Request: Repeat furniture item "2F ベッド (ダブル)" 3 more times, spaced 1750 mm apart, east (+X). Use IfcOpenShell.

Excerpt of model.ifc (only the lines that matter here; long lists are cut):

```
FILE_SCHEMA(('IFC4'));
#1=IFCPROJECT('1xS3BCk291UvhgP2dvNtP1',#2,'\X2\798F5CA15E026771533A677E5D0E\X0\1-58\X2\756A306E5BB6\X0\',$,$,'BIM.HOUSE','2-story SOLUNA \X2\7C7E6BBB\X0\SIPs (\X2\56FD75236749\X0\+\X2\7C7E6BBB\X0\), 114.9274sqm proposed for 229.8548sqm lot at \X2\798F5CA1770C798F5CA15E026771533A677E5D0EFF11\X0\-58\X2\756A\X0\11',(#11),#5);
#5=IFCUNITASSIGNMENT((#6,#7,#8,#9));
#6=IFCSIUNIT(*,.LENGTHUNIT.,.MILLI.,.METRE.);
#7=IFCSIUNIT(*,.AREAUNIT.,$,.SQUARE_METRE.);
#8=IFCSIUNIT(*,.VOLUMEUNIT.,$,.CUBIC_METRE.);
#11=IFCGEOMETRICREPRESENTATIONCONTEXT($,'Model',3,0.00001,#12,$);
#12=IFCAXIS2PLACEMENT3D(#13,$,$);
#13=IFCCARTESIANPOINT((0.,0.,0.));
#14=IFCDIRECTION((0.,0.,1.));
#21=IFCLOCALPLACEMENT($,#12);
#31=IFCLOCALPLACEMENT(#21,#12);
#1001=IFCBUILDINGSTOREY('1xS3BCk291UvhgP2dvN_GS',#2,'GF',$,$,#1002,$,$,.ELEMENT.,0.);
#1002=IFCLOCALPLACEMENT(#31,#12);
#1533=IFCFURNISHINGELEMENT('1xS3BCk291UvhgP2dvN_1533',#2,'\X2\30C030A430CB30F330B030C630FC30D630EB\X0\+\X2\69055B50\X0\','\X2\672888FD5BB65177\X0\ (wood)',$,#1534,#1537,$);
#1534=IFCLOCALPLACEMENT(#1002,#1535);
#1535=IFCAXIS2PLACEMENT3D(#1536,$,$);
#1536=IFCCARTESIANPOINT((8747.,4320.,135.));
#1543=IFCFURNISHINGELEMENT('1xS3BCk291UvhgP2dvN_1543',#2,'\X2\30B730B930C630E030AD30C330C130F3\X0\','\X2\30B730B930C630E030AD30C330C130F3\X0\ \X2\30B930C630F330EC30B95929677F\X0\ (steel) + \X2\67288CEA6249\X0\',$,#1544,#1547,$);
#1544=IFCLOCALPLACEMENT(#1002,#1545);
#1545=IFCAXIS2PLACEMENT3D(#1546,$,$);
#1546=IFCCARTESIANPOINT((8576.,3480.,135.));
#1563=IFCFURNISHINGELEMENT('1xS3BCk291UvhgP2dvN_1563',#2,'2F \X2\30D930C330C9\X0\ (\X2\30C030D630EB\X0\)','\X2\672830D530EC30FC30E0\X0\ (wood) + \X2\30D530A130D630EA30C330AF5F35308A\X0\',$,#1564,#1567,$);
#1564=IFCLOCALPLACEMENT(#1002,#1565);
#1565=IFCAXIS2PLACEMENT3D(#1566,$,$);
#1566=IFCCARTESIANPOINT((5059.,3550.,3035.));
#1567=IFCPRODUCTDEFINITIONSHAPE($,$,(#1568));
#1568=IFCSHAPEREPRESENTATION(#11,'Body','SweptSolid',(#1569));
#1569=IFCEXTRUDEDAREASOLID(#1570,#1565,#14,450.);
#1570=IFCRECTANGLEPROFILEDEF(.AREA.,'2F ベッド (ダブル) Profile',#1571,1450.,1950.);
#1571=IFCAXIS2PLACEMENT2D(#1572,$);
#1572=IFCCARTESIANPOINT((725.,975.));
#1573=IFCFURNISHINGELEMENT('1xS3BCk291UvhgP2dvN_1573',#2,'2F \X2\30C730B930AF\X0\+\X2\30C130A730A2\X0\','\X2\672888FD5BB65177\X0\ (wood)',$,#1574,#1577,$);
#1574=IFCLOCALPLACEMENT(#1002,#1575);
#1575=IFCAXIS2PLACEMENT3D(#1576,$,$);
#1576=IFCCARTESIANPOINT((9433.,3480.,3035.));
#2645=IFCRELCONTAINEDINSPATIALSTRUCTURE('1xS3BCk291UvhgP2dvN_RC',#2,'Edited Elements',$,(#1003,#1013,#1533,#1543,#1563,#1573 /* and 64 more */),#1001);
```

```python
import numpy as np
import ifcopenshell
import ifcopenshell.api.geometry
import ifcopenshell.api.root
import ifcopenshell.util.element
import ifcopenshell.util.placement
import ifcopenshell.util.unit

model = ifcopenshell.open("model.ifc")
unit_scale = ifcopenshell.util.unit.calculate_unit_scale(model)


def reuse_history(source, copy):
    """copy_class also copies each property set's owner history, people and application; keep the originals."""
    for rel in copy.IsDefinedBy:
        if rel.is_a("IfcRelDefinesByProperties") and (history := rel.RelatingPropertyDefinition.OwnerHistory):
            rel.RelatingPropertyDefinition.OwnerHistory = source.OwnerHistory
            ifcopenshell.util.element.remove_deep2(model, history)


source = model.by_id(1563)
base = ifcopenshell.util.placement.get_local_placement(source.ObjectPlacement)
step = np.array([1.0, 0.0, 0.0]) * 1.75 / unit_scale

for i in range(1, 4):
    copy = ifcopenshell.api.root.copy_class(model, product=source)
    copy.Representation = ifcopenshell.util.element.copy_deep(
        model, source.Representation, exclude=["IfcGeometricRepresentationContext", "IfcRepresentationMap"]
    )
    reuse_history(source, copy)
    matrix = base.copy()
    matrix[:3, 3] += i * step
    print("added at", matrix[:3, 3].round(3) + 0.0)
    ifcopenshell.api.geometry.edit_object_placement(model, product=copy, matrix=matrix, is_si=False)

model.write("model-out.ifc")
```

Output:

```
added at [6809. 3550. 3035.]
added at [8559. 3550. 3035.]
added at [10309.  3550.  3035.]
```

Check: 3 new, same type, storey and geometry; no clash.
